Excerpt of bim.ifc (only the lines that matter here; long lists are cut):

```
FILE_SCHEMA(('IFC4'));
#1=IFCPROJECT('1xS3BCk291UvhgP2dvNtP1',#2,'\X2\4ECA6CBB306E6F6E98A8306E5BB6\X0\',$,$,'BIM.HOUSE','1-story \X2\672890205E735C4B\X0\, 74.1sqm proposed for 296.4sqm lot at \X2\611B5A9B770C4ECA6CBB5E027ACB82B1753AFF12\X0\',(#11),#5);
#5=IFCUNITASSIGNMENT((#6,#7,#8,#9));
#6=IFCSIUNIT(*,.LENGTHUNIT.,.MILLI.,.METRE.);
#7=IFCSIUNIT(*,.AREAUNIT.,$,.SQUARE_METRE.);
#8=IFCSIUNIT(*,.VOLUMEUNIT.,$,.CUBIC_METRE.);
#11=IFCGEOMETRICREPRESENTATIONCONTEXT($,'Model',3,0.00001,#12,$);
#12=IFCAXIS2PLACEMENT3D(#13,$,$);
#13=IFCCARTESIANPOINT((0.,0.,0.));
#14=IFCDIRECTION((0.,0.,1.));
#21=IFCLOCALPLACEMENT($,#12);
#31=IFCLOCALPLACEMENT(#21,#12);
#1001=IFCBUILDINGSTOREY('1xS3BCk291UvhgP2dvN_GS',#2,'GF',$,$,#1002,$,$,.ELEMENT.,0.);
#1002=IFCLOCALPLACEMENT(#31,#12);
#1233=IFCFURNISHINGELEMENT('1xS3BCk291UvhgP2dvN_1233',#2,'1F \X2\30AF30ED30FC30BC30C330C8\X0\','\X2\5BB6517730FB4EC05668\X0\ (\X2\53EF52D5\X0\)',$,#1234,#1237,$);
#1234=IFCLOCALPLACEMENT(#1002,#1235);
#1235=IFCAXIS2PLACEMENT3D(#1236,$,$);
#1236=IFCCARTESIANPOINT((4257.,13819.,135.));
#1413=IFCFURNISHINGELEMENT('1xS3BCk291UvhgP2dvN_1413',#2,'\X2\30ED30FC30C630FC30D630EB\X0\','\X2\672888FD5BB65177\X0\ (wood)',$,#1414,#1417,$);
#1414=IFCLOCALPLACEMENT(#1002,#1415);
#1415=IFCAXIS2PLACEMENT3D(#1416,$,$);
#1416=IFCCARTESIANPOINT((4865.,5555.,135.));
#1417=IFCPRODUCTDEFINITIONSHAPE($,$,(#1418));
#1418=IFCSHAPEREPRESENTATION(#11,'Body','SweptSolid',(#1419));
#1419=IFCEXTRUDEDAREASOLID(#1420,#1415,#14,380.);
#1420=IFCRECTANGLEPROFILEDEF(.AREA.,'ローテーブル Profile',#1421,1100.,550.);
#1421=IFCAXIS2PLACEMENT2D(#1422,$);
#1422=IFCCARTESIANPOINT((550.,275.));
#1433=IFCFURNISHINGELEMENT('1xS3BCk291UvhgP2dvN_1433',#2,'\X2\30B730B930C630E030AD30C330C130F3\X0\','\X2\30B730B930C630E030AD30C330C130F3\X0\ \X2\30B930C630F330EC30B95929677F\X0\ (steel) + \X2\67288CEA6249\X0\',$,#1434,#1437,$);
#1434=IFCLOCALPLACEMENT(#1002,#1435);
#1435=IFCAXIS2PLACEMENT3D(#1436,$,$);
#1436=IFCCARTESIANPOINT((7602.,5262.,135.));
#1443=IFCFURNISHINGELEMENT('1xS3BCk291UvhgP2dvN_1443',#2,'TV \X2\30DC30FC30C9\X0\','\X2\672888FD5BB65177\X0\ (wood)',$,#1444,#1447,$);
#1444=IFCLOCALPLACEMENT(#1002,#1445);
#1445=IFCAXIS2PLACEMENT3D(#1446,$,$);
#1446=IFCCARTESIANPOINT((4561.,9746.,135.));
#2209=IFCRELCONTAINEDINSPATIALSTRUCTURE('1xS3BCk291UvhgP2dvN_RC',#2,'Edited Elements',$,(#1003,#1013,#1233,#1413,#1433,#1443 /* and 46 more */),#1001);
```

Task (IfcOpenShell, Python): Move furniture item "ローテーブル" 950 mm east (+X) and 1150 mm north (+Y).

```python
import ifcopenshell
import ifcopenshell.api.geometry
import ifcopenshell.util.placement

model = ifcopenshell.open("bim.ifc")

item = model.by_guid("1xS3BCk291UvhgP2dvN_1413")
matrix = ifcopenshell.util.placement.get_local_placement(item.ObjectPlacement)
matrix[0, 3] += 950.0
matrix[1, 3] += 1150.0
ifcopenshell.api.geometry.edit_object_placement(model, product=item, matrix=matrix, is_si=False)

print(ifcopenshell.util.placement.get_local_placement(item.ObjectPlacement).round(3) + 0.0)

model.write("bim_updated.ifc")
```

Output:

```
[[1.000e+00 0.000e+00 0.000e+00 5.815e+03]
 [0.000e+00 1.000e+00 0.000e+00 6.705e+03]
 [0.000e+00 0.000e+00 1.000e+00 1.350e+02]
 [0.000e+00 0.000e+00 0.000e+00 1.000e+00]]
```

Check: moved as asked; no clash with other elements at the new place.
